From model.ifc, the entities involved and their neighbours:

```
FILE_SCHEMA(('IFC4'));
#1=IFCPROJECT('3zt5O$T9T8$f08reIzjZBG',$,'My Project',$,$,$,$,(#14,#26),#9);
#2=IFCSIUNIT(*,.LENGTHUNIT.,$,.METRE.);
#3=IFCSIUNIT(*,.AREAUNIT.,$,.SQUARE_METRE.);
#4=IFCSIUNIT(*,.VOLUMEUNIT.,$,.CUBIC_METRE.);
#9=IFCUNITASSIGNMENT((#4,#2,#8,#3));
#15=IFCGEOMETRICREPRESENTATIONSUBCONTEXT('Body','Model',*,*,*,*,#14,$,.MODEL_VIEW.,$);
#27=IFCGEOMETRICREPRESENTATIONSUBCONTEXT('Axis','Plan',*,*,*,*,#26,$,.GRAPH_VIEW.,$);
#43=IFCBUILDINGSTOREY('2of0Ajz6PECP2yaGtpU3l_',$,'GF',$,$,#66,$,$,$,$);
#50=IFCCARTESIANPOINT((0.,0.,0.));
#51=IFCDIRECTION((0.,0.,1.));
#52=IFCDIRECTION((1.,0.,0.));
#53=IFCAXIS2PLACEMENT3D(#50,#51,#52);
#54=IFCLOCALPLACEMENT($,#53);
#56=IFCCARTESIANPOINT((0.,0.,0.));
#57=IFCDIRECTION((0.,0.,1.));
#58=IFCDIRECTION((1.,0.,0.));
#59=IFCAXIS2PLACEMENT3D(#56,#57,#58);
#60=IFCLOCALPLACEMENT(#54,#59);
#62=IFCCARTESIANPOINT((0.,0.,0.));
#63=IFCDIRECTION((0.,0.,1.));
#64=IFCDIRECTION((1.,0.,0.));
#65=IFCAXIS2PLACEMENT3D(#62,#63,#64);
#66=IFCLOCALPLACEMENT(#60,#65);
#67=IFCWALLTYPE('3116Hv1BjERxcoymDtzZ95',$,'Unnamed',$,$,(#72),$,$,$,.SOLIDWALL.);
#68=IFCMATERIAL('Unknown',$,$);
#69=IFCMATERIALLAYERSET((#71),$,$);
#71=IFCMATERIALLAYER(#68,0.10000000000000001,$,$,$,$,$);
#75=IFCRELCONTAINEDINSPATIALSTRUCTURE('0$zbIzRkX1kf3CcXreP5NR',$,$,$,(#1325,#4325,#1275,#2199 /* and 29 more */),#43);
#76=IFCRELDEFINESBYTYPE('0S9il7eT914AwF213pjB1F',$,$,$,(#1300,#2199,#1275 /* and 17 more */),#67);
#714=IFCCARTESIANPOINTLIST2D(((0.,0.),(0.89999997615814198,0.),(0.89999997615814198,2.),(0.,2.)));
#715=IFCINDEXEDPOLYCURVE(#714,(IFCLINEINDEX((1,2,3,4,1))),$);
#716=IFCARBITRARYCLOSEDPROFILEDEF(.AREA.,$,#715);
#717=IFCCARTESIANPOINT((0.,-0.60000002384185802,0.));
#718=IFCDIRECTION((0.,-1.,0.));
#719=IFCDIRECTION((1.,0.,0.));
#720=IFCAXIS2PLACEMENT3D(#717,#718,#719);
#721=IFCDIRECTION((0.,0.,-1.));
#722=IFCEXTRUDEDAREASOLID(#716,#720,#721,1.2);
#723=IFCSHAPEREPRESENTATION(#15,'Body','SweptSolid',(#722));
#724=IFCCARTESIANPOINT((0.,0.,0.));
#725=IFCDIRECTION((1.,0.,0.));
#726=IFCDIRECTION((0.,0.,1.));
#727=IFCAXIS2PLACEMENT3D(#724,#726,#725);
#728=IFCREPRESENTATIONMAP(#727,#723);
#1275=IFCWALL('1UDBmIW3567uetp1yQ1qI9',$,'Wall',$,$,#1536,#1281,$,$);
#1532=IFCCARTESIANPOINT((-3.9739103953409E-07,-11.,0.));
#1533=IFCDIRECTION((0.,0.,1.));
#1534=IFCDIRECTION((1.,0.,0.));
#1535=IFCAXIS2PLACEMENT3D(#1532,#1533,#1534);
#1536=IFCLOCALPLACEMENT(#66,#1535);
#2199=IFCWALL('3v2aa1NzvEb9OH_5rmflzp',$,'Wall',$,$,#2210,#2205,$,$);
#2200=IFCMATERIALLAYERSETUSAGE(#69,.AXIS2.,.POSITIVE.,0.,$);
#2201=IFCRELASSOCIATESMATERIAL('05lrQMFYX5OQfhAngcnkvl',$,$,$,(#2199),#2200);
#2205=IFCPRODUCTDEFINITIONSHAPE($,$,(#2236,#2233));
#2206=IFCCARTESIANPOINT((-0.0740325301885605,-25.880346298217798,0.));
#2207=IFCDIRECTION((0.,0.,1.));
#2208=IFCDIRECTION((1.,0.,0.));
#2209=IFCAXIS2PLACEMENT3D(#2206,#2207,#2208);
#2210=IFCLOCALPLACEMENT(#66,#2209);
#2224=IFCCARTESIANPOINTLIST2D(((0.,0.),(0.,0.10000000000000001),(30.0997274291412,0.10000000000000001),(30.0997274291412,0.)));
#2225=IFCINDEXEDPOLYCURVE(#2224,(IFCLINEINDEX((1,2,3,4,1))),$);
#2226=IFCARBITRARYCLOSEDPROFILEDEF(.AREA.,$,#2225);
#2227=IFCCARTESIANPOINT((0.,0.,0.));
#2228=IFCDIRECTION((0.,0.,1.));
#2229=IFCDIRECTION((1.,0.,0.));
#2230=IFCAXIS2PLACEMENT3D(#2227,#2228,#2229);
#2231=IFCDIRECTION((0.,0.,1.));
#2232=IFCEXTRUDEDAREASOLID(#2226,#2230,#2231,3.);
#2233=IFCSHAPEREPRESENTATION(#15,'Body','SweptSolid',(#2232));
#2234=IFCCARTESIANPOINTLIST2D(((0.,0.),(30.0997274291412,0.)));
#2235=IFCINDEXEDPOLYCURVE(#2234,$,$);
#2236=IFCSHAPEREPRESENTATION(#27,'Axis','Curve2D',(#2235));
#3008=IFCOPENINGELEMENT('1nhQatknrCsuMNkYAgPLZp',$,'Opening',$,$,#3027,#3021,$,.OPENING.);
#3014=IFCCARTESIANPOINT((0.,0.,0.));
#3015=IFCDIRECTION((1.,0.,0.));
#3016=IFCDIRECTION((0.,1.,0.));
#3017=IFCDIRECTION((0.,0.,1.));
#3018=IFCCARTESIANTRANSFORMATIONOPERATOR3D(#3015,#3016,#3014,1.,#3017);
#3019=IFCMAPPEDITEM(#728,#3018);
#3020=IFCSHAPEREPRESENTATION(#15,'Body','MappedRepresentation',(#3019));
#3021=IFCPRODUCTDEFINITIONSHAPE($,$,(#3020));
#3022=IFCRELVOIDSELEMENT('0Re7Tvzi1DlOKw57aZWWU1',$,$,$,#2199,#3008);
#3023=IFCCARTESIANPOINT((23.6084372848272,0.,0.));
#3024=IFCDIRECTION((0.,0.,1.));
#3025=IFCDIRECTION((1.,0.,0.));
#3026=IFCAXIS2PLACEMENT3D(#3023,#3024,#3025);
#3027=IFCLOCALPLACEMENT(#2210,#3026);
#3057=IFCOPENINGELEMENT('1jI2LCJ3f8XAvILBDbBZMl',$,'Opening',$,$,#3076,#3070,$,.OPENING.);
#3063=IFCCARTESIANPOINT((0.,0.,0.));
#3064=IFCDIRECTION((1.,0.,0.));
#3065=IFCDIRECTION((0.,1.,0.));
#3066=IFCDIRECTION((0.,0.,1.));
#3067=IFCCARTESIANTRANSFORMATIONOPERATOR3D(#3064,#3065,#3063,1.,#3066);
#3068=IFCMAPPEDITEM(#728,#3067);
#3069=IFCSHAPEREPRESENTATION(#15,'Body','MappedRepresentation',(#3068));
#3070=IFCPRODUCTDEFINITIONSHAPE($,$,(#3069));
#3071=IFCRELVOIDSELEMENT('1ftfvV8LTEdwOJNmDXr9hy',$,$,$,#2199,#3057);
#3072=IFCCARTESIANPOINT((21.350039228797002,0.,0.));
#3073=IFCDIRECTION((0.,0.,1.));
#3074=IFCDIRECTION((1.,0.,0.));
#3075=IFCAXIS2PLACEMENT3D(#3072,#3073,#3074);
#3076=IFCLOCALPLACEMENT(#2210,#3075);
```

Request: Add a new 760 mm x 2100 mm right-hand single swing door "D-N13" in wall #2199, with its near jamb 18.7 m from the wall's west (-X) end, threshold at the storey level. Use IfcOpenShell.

```python
import numpy as np
import ifcopenshell
import ifcopenshell.api.feature
import ifcopenshell.api.geometry
import ifcopenshell.api.root
import ifcopenshell.api.spatial
import ifcopenshell.geom
import ifcopenshell.util.element
import ifcopenshell.util.placement
import ifcopenshell.util.representation
import ifcopenshell.util.shape
import ifcopenshell.util.unit

model = ifcopenshell.open("model.ifc")
unit_scale = ifcopenshell.util.unit.calculate_unit_scale(model)
settings = ifcopenshell.geom.settings()


def volume(element):
    """Net volume in cubic metres, openings subtracted."""
    shape = ifcopenshell.geom.create_shape(settings, element)
    return ifcopenshell.util.shape.get_volume(shape.geometry)


wall = model.by_guid("3v2aa1NzvEb9OH_5rmflzp")
storey = ifcopenshell.util.element.get_container(wall, ifc_class="IfcBuildingStorey")
context = ifcopenshell.util.representation.get_context(model, "Model", "Body", "MODEL_VIEW")
before = volume(wall)

width, height, from_end, sill = 0.76, 2.1, 18.7, 0.0  # metres

# The wall runs along its own X axis, and the end named is its -X end.
wall_shape = ifcopenshell.geom.create_shape(settings, wall)
x, y, z = ifcopenshell.util.shape.get_vertices(wall_shape.geometry).T
start = x.min() + from_end
face, thickness = float(y.min()), float(y.max() - y.min())
wall_matrix = ifcopenshell.util.placement.get_local_placement(wall.ObjectPlacement)
level = ifcopenshell.util.placement.get_local_placement(storey.ObjectPlacement)[2, 3]


def in_wall(x, y):
    """Placement at x, y metres in the wall's axes, at sill height."""
    matrix = wall_matrix.copy()
    matrix[:, 3] = wall_matrix @ np.array([x / unit_scale, y / unit_scale, 0.0, 1.0])
    matrix[2, 3] = level + sill / unit_scale
    return matrix


# Opening: a box that overshoots both wall faces by 50 mm.
opening = ifcopenshell.api.root.create_entity(model, ifc_class="IfcOpeningElement", predefined_type="OPENING")
box = ifcopenshell.api.geometry.add_wall_representation(
    model, context=context, length=width, height=height, thickness=thickness + 0.1
)
ifcopenshell.api.geometry.assign_representation(model, product=opening, representation=box)
ifcopenshell.api.geometry.edit_object_placement(model, product=opening, matrix=in_wall(start, face - 0.05), is_si=False)
ifcopenshell.api.feature.add_feature(model, feature=opening, element=wall)

door = ifcopenshell.api.root.create_entity(model, ifc_class="IfcDoor", name="D-N13", predefined_type="DOOR")
door.OverallWidth, door.OverallHeight = width / unit_scale, height / unit_scale
door.OperationType = "SINGLE_SWING_RIGHT"
body = ifcopenshell.api.geometry.add_door_representation(
    model,
    context=context,
    overall_width=door.OverallWidth,
    overall_height=door.OverallHeight,
    operation_type="SINGLE_SWING_RIGHT",
    lining_properties={"LiningDepth": thickness / unit_scale, "ThresholdDepth": thickness / unit_scale},
)
ifcopenshell.api.geometry.assign_representation(model, product=door, representation=body)
ifcopenshell.api.spatial.assign_container(model, products=[door], relating_structure=storey)
ifcopenshell.api.feature.add_filling(model, opening=opening, element=door)

# The lining spans the wall, so the door starts at the wall face.
ifcopenshell.api.geometry.edit_object_placement(model, product=door, matrix=in_wall(start, face), is_si=False)

after = volume(wall)

print(f"wall volume {before:.3f} -> {after:.3f} m3")

model.write("model_v2.ifc")
```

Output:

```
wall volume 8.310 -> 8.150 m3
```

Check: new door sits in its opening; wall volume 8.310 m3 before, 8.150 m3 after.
